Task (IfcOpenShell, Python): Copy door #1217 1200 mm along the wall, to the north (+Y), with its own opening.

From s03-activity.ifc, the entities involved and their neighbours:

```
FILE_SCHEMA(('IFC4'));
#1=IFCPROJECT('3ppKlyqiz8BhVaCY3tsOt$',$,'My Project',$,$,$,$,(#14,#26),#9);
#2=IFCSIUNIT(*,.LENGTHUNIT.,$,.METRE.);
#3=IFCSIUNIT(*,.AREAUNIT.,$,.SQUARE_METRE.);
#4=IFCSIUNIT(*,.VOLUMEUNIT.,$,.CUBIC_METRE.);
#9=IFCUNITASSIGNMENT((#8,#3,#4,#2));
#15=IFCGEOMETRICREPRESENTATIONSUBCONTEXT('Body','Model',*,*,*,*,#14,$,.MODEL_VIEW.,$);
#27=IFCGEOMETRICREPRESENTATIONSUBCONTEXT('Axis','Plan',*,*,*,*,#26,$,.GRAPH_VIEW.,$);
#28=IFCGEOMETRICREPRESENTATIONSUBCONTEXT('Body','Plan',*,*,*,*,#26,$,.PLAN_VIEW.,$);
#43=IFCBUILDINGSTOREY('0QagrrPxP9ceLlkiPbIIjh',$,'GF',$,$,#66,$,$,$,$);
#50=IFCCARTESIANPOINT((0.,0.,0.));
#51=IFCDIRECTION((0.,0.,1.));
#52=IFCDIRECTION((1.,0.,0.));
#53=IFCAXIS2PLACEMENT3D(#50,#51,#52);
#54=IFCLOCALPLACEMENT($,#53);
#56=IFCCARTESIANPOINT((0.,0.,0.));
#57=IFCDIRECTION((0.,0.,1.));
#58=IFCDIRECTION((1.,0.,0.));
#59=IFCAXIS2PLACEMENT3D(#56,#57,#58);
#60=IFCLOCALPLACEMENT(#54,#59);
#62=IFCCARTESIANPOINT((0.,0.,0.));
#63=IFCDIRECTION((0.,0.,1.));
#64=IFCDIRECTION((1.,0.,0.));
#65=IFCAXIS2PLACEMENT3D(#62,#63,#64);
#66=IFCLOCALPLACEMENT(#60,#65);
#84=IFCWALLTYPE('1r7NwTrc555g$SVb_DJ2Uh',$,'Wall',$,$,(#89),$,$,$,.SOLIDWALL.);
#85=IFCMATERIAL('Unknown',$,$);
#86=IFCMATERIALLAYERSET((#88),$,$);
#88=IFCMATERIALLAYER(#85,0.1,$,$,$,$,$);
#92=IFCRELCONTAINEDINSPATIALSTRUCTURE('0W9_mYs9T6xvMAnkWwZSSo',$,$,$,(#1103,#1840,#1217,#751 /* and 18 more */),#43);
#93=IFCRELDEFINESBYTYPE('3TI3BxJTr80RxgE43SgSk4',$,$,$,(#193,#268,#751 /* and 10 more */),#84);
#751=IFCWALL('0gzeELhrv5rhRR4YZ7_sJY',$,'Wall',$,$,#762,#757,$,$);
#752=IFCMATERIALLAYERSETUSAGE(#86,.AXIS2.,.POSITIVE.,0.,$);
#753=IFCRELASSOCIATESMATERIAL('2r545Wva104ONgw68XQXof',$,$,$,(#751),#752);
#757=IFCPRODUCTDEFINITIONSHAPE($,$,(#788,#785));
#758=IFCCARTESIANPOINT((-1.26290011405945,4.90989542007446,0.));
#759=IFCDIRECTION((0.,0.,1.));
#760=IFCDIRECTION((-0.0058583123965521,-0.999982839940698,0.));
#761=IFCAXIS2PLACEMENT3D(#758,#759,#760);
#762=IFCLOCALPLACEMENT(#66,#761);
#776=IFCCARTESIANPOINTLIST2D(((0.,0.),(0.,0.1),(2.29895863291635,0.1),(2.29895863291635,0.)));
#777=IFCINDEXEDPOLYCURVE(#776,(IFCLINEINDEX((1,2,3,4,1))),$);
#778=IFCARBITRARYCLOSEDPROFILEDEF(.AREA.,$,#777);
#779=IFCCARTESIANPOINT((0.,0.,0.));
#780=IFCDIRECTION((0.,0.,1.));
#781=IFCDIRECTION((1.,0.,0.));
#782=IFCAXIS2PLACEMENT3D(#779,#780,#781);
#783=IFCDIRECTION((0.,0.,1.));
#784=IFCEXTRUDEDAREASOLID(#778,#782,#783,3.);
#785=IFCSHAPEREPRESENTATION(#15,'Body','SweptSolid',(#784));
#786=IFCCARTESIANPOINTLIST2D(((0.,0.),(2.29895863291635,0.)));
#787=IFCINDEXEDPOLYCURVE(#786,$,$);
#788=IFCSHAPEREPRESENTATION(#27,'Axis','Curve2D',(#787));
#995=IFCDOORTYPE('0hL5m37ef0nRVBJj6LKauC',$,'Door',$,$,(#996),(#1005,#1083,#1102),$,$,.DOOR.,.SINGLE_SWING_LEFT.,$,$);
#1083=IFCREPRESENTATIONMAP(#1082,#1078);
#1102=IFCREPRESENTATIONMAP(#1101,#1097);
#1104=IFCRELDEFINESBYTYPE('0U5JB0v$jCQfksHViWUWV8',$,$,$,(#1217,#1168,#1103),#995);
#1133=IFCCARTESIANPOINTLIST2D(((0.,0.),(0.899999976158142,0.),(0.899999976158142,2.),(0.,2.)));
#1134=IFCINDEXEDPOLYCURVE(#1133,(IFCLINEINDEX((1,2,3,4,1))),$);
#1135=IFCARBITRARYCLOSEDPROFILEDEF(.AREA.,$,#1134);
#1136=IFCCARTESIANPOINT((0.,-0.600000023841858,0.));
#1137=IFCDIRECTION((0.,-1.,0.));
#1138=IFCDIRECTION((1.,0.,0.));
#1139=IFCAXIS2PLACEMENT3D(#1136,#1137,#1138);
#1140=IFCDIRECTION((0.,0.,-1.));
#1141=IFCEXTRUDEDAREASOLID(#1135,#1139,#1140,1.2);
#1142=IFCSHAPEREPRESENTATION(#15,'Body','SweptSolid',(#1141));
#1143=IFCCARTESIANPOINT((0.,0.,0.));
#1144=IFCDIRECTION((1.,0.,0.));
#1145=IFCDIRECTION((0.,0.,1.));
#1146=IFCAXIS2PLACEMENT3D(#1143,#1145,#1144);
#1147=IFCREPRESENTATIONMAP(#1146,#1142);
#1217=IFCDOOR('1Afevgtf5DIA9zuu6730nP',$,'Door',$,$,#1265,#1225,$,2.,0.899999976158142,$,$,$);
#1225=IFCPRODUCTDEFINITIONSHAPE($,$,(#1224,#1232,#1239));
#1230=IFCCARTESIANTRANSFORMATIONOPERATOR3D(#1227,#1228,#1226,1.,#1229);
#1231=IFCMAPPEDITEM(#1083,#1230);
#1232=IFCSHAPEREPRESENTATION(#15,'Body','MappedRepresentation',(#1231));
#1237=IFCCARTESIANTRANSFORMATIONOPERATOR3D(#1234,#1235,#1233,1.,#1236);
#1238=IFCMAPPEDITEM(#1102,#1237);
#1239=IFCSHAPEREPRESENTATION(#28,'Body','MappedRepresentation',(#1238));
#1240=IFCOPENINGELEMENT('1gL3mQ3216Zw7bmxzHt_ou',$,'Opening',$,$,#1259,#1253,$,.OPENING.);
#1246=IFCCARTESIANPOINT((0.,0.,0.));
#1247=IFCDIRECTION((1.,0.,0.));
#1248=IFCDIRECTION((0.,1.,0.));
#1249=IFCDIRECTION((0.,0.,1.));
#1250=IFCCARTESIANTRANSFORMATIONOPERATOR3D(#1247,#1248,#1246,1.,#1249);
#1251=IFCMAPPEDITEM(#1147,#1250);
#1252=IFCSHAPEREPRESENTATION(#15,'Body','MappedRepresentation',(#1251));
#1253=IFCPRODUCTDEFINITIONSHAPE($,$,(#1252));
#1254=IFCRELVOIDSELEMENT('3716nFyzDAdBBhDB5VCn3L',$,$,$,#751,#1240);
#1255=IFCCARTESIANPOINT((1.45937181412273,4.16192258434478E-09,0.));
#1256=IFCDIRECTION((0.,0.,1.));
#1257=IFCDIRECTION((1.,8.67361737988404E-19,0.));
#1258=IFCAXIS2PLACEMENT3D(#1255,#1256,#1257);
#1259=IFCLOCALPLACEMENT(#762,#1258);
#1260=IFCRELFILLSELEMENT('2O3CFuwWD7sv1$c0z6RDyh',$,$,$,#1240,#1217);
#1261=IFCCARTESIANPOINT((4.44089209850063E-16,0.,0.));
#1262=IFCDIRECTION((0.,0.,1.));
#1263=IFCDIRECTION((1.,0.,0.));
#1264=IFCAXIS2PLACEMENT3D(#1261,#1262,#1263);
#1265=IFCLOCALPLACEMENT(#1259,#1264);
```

```python
import ifcopenshell
import ifcopenshell.api.feature
import ifcopenshell.api.geometry
import ifcopenshell.api.root
import ifcopenshell.geom
import ifcopenshell.util.element
import ifcopenshell.util.placement
import ifcopenshell.util.shape

model = ifcopenshell.open("s03-activity.ifc")
settings = ifcopenshell.geom.settings()


def volume(element):
    """Net volume in cubic metres, openings subtracted."""
    shape = ifcopenshell.geom.create_shape(settings, element)
    return ifcopenshell.util.shape.get_volume(shape.geometry)


door = model.by_guid("1Afevgtf5DIA9zuu6730nP")
opening = door.FillsVoids[0].RelatingOpeningElement
wall = opening.VoidsElements[0].RelatingBuildingElement
before = volume(wall)
shift = ifcopenshell.util.placement.get_local_placement(wall.ObjectPlacement)[:3, 0] * -1.2

# copy_class copies the void relationship, type, container and properties, but no geometry.
new_opening = ifcopenshell.api.root.copy_class(model, product=opening)
new_opening.Representation = ifcopenshell.util.element.copy_deep(
    model, opening.Representation, exclude=["IfcGeometricRepresentationContext", "IfcRepresentationMap"]
)
new_door = ifcopenshell.api.root.copy_class(model, product=door)
new_door.Representation = ifcopenshell.util.element.copy_deep(
    model, door.Representation, exclude=["IfcGeometricRepresentationContext", "IfcRepresentationMap"]
)
ifcopenshell.api.feature.add_filling(model, opening=new_opening, element=new_door)

for old, new in ((opening, new_opening), (door, new_door)):
    matrix = ifcopenshell.util.placement.get_local_placement(old.ObjectPlacement)
    matrix[:3, 3] += shift
    ifcopenshell.api.geometry.edit_object_placement(model, product=new, matrix=matrix, is_si=False)

after = volume(wall)

print(f"wall volume {before:.3f} -> {after:.3f} m3")

model.write("s03-activity_rev.ifc")
```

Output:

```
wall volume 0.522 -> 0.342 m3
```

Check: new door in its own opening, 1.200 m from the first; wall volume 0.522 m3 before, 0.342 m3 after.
